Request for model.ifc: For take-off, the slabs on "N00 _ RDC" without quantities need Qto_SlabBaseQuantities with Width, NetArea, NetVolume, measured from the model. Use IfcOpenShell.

First a look at what the model holds.

```python
import ifcopenshell
import ifcopenshell.util.element
import ifcopenshell.util.unit

model = ifcopenshell.open("model.ifc")
print(model.schema)
for unit_type in ("LENGTHUNIT", "AREAUNIT", "VOLUMEUNIT"):
    print(unit_type, ifcopenshell.util.unit.calculate_unit_scale(model, unit_type))
storey = next(s for s in model.by_type("IfcBuildingStorey") if s.Name == "N00 _ RDC")
slabs = [e for e in ifcopenshell.util.element.get_decomposition(storey) if e.is_a("IfcSlab")]
for e in sorted(slabs, key=lambda e: e.id()):
    print(e.id(), e.is_a(), e.Name, list(ifcopenshell.util.element.get_psets(e, qtos_only=True)), sep=" | ")
```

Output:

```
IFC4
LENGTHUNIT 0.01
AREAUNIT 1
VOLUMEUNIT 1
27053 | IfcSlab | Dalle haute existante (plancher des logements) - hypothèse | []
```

```python
import ifcopenshell
import ifcopenshell.api.pset
import ifcopenshell.geom
import ifcopenshell.util.element
import ifcopenshell.util.shape
import ifcopenshell.util.unit

model = ifcopenshell.open("model.ifc")
unit_scale = ifcopenshell.util.unit.calculate_unit_scale(model)
area_scale = ifcopenshell.util.unit.calculate_unit_scale(model, "AREAUNIT")
volume_scale = ifcopenshell.util.unit.calculate_unit_scale(model, "VOLUMEUNIT")
settings = ifcopenshell.geom.settings()

storey = next(s for s in model.by_type("IfcBuildingStorey") if s.Name == "N00 _ RDC")
slabs = [e for e in ifcopenshell.util.element.get_decomposition(storey) if e.is_a("IfcSlab")]

for e in sorted(slabs, key=lambda e: e.id()):
    if ifcopenshell.util.element.get_psets(e, qtos_only=True, should_inherit=False):
        continue
    # Geometry comes back in metres, in the element's own axes.
    shape = ifcopenshell.geom.create_shape(settings, e)
    values = {
        "Width": ifcopenshell.util.shape.get_z(shape.geometry) / unit_scale,
        "NetArea": ifcopenshell.util.shape.get_footprint_area(shape.geometry) / area_scale,
        "NetVolume": ifcopenshell.util.shape.get_volume(shape.geometry) / volume_scale,
    }
    qto = ifcopenshell.api.pset.add_qto(model, product=e, name="Qto_SlabBaseQuantities")
    ifcopenshell.api.pset.edit_qto(model, qto=qto, properties=values)
    print(e.id(), {k: round(v, 3) for k, v in values.items()})

model.write("model-out.ifc")
```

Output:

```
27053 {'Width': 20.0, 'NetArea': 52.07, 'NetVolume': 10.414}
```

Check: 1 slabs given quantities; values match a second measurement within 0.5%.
